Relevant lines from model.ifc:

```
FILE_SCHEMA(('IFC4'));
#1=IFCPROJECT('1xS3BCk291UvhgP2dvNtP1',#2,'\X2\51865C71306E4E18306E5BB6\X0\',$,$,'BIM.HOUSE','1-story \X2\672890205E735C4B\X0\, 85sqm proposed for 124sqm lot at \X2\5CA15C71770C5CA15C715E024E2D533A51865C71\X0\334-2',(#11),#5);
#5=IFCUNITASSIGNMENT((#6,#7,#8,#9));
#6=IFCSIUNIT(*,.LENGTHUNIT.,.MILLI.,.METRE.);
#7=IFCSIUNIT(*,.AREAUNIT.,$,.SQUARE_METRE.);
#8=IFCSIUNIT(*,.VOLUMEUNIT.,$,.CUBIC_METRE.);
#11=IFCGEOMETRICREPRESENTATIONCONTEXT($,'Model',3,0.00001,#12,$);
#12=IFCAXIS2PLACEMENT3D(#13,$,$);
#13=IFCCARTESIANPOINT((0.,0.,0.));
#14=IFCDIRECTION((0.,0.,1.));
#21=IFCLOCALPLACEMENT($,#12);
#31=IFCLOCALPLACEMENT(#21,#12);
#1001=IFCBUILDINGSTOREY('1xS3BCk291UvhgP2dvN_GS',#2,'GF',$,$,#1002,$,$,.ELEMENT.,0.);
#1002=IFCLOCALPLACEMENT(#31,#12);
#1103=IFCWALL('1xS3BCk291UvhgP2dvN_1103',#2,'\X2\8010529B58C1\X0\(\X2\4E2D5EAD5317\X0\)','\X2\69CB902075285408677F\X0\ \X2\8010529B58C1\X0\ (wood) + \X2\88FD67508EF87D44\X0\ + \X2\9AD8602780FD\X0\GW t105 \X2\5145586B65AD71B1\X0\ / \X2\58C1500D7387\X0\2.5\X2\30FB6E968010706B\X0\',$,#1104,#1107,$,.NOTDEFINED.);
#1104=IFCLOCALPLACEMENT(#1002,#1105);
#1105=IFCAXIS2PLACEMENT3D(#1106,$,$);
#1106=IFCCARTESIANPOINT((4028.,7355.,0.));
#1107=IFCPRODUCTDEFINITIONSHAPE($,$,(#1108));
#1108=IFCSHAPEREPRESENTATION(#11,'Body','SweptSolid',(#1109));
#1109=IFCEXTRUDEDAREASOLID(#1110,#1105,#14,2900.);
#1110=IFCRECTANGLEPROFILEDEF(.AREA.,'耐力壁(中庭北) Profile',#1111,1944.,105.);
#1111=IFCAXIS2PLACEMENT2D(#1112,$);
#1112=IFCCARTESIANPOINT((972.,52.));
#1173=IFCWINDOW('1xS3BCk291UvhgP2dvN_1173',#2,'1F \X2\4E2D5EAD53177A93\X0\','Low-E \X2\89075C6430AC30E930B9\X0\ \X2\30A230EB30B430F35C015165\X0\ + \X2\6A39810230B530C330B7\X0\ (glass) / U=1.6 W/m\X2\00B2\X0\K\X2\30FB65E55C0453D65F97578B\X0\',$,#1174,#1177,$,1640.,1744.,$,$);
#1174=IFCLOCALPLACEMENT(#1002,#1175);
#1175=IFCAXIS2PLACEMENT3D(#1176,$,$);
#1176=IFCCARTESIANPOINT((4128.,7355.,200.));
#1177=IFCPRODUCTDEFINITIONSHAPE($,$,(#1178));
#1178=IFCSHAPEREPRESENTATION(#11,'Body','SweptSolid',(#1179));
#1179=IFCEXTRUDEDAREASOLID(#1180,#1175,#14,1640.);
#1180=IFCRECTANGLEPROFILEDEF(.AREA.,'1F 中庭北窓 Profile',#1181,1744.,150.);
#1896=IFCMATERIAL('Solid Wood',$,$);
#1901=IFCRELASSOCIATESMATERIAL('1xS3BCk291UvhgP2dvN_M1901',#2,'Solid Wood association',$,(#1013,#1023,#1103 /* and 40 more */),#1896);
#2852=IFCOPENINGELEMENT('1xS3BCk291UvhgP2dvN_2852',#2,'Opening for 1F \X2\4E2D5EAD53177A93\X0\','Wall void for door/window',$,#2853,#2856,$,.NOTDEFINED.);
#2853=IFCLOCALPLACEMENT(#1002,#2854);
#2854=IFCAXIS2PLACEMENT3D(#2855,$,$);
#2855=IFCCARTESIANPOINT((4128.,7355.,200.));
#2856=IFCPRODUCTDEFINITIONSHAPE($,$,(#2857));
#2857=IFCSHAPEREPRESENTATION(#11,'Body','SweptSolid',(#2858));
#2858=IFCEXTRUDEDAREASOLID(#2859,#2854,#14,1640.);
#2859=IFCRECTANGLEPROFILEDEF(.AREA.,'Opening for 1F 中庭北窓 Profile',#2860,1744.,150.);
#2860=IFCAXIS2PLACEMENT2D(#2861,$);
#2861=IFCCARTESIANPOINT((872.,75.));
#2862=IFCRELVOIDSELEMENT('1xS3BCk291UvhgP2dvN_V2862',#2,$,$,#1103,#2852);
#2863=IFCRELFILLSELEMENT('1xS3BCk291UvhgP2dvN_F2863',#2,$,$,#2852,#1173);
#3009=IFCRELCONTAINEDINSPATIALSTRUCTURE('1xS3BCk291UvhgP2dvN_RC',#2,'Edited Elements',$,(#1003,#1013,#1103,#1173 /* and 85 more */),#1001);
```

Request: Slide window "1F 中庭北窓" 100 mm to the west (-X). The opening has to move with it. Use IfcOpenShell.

```python
import ifcopenshell
import ifcopenshell.api.geometry
import ifcopenshell.util.placement
import ifcopenshell.util.unit

model = ifcopenshell.open("model.ifc")
unit_scale = ifcopenshell.util.unit.calculate_unit_scale(model)

window = model.by_id(1173)
opening = window.FillsVoids[0].RelatingOpeningElement
wall = opening.VoidsElements[0].RelatingBuildingElement

wall_matrix = ifcopenshell.util.placement.get_local_placement(wall.ObjectPlacement)
shift = wall_matrix[:3, 0] * -0.1 / unit_scale
before = ifcopenshell.util.placement.get_local_placement(window.ObjectPlacement)[:3, 3].copy()

# The window is not placed relative to its opening, so move both.
for product in (opening, window):
    matrix = ifcopenshell.util.placement.get_local_placement(product.ObjectPlacement)
    matrix[:3, 3] += shift
    ifcopenshell.api.geometry.edit_object_placement(model, product=product, matrix=matrix, is_si=False)

after = ifcopenshell.util.placement.get_local_placement(window.ObjectPlacement)[:3, 3]
print("window moved by", (after - before).round(3) + 0.0)

model.write("model_updated.ifc")
```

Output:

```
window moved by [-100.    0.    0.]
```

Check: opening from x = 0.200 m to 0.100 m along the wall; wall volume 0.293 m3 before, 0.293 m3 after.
